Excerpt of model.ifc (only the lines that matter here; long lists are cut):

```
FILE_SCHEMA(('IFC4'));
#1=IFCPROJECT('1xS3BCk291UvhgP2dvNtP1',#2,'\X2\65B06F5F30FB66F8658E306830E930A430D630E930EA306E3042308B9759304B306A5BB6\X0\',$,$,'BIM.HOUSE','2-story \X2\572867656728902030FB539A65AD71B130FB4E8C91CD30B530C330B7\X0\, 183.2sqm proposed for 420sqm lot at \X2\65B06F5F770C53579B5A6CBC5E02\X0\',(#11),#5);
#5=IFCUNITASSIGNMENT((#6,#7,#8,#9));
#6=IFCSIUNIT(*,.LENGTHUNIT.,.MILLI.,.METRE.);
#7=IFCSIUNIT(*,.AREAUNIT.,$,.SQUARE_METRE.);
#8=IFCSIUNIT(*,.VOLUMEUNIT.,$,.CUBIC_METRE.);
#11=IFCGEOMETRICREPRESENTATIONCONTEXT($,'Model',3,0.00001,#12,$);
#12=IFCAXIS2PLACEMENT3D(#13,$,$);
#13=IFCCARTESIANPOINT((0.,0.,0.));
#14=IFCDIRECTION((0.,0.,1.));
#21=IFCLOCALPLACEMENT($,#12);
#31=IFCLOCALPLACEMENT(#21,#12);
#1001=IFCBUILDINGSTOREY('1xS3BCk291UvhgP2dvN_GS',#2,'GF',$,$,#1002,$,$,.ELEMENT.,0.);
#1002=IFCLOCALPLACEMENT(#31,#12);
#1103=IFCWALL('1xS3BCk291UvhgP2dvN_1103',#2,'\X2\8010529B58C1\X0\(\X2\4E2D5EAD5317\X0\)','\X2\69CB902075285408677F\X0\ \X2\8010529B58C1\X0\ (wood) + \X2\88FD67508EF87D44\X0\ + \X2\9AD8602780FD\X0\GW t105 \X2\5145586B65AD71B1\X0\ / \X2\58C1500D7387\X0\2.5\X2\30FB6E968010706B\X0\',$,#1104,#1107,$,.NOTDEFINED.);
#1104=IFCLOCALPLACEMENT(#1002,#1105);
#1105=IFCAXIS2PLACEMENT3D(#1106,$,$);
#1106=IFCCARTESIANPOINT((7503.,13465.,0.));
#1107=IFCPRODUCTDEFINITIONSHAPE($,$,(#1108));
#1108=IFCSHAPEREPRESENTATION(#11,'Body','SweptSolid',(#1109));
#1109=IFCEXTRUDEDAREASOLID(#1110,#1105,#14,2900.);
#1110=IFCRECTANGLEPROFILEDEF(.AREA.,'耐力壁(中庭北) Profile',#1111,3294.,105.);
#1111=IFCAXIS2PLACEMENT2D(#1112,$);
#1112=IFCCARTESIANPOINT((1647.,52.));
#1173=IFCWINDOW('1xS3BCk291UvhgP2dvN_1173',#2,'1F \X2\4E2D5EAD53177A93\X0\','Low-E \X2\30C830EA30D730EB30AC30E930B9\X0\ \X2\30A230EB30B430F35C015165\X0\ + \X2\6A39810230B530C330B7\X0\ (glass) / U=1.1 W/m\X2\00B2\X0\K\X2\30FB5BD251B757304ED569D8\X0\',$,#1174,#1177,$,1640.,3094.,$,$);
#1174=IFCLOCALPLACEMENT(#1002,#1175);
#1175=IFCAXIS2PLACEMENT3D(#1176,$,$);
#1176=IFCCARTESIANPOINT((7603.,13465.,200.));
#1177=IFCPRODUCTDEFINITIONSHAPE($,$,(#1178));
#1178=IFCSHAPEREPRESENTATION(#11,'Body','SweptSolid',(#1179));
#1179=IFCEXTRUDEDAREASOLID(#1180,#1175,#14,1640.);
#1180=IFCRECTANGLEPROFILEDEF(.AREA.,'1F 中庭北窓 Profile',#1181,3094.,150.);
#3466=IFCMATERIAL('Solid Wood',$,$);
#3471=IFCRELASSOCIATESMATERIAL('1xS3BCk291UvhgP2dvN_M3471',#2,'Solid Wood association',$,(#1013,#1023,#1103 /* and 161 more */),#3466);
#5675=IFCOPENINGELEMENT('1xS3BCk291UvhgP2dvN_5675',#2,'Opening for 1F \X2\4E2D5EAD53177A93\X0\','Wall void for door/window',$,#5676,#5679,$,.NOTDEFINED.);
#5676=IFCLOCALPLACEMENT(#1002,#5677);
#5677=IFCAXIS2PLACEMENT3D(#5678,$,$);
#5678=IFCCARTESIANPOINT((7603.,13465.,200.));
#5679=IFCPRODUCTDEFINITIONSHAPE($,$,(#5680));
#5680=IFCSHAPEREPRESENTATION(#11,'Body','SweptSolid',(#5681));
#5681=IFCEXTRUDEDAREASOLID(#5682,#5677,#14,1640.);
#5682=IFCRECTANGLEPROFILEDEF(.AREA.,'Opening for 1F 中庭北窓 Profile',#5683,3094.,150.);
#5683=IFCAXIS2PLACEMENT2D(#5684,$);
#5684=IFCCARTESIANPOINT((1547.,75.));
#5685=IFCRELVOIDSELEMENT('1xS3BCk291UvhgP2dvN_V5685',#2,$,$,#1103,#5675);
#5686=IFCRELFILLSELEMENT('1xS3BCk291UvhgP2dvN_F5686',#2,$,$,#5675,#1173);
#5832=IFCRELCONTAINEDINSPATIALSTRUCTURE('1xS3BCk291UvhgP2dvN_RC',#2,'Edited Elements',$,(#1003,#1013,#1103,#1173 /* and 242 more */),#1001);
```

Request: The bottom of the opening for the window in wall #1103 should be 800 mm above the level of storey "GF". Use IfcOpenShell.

```python
import numpy as np
import ifcopenshell
import ifcopenshell.api.geometry
import ifcopenshell.geom
import ifcopenshell.util.element
import ifcopenshell.util.placement
import ifcopenshell.util.shape
import ifcopenshell.util.unit

model = ifcopenshell.open("model.ifc")
unit_scale = ifcopenshell.util.unit.calculate_unit_scale(model)

window = model.by_id(1173)
opening = window.FillsVoids[0].RelatingOpeningElement
storey = ifcopenshell.util.element.get_container(window, ifc_class="IfcBuildingStorey")
level = ifcopenshell.util.placement.get_local_placement(storey.ObjectPlacement)[2, 3]

# The opening's origin need not be at the sill, so measure its lowest point.
shape = ifcopenshell.geom.create_shape(ifcopenshell.geom.settings(), opening)
bottom = ifcopenshell.util.shape.get_shape_bottom_elevation(shape, shape.geometry) / unit_scale
dz = level + 800.0 - bottom

shift = np.array([0.0, 0.0, dz])
# The window is not placed relative to its opening, so move both.
for product in (opening, window):
    matrix = ifcopenshell.util.placement.get_local_placement(product.ObjectPlacement)
    matrix[:3, 3] += shift
    ifcopenshell.api.geometry.edit_object_placement(model, product=product, matrix=matrix, is_si=False)

print(f"moved by {dz * unit_scale:+.3f} m")

model.write("model_v2.ifc")
```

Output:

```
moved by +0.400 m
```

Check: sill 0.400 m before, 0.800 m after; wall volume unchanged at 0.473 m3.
